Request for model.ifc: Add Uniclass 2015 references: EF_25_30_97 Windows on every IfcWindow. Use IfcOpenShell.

First a look at what the model holds.

```python
import ifcopenshell

model = ifcopenshell.open("model.ifc")
print(model.schema)
print("classifications:", [c.Name for c in model.by_type("IfcClassification")])
for ifc_class in ("IfcDoor", "IfcRoof", "IfcStair", "IfcWall", "IfcWindow"):
    print(ifc_class, len(model.by_type(ifc_class)))
```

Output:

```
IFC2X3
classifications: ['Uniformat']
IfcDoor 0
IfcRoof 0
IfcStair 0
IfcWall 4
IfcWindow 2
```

```python
import ifcopenshell
import ifcopenshell.api.classification

model = ifcopenshell.open("model.ifc")

# IFC2X3 requires Source and Edition and has no link from the project to the system.
system = model.create_entity("IfcClassification", Source="NBS", Edition="2015", Name="Uniclass 2015")

codes = {
    "IfcWindow": ("EF_25_30_97", "Windows"),
}
for ifc_class, (code, name) in codes.items():
    products = model.by_type(ifc_class)
    ifcopenshell.api.classification.add_reference(
        model, products=products, classification=system, identification=code, name=name
    )
    print(code, len(products))

model.write("model-out.ifc")
```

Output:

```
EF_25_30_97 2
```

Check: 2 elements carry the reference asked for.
